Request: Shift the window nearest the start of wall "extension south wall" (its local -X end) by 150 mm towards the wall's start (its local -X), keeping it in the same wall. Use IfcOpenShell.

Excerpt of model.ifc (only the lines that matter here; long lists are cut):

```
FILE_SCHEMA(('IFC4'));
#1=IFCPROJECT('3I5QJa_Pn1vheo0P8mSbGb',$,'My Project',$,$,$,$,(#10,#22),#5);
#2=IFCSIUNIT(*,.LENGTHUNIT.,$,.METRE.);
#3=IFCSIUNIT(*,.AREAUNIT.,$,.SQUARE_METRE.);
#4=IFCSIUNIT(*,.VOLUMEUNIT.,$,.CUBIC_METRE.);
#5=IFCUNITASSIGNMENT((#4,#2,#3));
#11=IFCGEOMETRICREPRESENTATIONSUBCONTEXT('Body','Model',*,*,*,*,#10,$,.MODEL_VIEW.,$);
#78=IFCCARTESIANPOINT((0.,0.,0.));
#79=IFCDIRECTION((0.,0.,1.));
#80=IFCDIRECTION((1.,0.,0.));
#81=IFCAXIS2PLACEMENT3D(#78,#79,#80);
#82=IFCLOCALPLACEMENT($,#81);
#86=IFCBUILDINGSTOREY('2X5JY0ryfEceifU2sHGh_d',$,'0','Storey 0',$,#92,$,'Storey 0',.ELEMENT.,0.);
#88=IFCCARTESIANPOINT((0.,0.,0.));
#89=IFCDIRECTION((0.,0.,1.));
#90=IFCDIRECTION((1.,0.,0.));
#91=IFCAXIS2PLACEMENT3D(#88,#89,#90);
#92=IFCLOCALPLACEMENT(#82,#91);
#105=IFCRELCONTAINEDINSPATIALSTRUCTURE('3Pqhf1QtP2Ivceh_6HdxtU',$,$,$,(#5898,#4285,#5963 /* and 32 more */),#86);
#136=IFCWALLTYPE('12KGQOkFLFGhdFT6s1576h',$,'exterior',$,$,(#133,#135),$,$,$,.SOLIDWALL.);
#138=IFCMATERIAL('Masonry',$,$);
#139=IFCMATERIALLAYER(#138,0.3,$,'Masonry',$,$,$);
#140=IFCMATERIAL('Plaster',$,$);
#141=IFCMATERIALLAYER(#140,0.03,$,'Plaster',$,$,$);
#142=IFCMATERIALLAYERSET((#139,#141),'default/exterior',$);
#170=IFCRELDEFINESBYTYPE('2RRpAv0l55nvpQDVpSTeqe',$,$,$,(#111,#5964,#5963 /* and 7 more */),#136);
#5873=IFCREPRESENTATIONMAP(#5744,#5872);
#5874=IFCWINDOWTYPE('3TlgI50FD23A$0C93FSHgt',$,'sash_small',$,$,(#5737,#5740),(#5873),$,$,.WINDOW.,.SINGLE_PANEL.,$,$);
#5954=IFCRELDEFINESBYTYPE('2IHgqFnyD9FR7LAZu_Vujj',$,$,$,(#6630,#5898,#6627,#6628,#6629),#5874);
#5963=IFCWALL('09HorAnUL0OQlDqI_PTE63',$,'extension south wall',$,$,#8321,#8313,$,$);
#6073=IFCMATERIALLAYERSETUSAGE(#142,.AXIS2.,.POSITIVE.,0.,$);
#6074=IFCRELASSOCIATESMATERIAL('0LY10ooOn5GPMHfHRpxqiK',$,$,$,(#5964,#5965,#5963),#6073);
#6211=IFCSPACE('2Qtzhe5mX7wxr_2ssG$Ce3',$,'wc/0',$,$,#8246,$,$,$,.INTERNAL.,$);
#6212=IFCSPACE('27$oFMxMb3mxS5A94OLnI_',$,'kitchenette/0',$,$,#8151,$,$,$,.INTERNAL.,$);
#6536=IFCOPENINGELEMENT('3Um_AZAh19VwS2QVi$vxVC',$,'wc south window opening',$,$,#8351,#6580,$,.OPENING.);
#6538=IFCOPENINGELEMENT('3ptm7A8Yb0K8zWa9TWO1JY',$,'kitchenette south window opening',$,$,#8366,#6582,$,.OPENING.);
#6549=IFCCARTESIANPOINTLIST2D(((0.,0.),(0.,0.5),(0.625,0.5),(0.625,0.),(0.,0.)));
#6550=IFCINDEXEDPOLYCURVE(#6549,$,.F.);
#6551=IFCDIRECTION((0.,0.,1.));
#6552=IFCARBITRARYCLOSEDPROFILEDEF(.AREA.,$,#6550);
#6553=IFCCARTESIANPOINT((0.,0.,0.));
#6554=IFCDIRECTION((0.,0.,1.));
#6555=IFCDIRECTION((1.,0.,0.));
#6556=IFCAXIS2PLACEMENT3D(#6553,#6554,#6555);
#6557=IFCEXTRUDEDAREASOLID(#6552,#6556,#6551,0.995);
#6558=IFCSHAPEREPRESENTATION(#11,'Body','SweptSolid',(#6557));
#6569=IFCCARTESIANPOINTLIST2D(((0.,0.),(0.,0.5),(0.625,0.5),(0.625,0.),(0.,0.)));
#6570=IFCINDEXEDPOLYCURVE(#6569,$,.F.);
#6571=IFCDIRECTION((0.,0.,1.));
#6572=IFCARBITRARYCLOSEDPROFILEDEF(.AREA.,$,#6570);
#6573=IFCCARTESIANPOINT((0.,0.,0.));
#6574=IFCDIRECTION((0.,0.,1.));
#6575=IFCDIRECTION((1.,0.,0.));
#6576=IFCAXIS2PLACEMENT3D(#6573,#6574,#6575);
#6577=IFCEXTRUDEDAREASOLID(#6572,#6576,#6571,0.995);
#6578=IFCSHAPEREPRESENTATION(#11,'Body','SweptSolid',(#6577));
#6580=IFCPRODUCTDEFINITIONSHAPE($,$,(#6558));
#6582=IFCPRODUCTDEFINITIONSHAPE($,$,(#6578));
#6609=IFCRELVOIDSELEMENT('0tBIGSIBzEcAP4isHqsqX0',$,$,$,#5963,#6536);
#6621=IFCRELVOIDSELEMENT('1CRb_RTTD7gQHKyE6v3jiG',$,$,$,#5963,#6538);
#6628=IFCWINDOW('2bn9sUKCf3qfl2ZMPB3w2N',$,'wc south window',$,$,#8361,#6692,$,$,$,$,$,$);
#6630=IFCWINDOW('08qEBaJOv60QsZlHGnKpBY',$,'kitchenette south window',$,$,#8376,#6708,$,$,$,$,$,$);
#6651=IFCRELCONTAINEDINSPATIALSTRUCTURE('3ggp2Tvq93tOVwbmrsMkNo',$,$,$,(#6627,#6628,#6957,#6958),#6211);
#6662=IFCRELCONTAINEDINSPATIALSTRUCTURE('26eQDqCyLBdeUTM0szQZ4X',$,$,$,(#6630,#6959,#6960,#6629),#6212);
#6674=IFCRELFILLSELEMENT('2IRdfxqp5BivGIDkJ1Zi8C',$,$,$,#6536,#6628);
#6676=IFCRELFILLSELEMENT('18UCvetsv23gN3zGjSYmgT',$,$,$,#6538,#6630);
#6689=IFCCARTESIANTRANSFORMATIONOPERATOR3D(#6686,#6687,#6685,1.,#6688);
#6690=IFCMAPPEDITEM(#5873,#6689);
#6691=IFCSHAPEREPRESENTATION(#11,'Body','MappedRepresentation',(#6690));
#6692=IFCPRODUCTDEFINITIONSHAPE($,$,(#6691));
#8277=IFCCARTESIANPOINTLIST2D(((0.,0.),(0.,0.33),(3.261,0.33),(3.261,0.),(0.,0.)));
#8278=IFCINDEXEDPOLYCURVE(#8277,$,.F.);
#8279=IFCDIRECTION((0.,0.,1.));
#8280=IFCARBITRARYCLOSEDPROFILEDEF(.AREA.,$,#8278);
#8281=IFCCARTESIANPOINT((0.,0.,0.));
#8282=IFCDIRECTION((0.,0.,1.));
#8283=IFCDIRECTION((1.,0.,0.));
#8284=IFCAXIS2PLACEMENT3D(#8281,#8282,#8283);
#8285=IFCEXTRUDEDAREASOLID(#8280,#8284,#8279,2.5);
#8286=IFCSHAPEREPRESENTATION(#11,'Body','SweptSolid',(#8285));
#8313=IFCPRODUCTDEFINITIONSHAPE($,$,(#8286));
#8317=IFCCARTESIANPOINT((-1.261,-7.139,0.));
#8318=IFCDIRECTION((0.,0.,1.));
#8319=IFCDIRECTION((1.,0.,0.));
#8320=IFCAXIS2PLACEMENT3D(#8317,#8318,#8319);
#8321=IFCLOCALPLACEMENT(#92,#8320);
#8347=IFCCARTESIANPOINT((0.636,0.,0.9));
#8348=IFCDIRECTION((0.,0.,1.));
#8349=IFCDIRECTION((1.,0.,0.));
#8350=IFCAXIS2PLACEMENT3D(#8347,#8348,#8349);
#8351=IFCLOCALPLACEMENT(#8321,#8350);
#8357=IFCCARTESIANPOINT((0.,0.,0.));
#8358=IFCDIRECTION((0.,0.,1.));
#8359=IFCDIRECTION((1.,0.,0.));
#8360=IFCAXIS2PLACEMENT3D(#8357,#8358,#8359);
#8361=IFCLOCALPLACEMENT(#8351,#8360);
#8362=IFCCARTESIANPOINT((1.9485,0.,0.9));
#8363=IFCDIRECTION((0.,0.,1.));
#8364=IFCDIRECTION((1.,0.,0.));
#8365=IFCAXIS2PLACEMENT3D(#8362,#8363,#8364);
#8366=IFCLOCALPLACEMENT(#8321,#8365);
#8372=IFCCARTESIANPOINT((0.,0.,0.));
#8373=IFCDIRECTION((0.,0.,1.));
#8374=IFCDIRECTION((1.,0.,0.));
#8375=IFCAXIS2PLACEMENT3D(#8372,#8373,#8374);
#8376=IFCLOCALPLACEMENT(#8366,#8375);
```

```python
import ifcopenshell
import ifcopenshell.api.geometry
import ifcopenshell.util.placement
import ifcopenshell.util.unit

model = ifcopenshell.open("model.ifc")
unit_scale = ifcopenshell.util.unit.calculate_unit_scale(model)

window = model.by_id(6628)
opening = window.FillsVoids[0].RelatingOpeningElement
wall = opening.VoidsElements[0].RelatingBuildingElement

wall_matrix = ifcopenshell.util.placement.get_local_placement(wall.ObjectPlacement)
shift = wall_matrix[:3, 0] * -0.15 / unit_scale
before = ifcopenshell.util.placement.get_local_placement(window.ObjectPlacement)[:3, 3].copy()

# The window is placed relative to its opening, so it follows when the opening moves.
matrix = ifcopenshell.util.placement.get_local_placement(opening.ObjectPlacement)
matrix[:3, 3] += shift
ifcopenshell.api.geometry.edit_object_placement(
    model, product=opening, matrix=matrix, is_si=False, should_transform_children=True
)

after = ifcopenshell.util.placement.get_local_placement(window.ObjectPlacement)[:3, 3]
print("window moved by", (after - before).round(3) + 0.0)

model.write("model_v2.ifc")
```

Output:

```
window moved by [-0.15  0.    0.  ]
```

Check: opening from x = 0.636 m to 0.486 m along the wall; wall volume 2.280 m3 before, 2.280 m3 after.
